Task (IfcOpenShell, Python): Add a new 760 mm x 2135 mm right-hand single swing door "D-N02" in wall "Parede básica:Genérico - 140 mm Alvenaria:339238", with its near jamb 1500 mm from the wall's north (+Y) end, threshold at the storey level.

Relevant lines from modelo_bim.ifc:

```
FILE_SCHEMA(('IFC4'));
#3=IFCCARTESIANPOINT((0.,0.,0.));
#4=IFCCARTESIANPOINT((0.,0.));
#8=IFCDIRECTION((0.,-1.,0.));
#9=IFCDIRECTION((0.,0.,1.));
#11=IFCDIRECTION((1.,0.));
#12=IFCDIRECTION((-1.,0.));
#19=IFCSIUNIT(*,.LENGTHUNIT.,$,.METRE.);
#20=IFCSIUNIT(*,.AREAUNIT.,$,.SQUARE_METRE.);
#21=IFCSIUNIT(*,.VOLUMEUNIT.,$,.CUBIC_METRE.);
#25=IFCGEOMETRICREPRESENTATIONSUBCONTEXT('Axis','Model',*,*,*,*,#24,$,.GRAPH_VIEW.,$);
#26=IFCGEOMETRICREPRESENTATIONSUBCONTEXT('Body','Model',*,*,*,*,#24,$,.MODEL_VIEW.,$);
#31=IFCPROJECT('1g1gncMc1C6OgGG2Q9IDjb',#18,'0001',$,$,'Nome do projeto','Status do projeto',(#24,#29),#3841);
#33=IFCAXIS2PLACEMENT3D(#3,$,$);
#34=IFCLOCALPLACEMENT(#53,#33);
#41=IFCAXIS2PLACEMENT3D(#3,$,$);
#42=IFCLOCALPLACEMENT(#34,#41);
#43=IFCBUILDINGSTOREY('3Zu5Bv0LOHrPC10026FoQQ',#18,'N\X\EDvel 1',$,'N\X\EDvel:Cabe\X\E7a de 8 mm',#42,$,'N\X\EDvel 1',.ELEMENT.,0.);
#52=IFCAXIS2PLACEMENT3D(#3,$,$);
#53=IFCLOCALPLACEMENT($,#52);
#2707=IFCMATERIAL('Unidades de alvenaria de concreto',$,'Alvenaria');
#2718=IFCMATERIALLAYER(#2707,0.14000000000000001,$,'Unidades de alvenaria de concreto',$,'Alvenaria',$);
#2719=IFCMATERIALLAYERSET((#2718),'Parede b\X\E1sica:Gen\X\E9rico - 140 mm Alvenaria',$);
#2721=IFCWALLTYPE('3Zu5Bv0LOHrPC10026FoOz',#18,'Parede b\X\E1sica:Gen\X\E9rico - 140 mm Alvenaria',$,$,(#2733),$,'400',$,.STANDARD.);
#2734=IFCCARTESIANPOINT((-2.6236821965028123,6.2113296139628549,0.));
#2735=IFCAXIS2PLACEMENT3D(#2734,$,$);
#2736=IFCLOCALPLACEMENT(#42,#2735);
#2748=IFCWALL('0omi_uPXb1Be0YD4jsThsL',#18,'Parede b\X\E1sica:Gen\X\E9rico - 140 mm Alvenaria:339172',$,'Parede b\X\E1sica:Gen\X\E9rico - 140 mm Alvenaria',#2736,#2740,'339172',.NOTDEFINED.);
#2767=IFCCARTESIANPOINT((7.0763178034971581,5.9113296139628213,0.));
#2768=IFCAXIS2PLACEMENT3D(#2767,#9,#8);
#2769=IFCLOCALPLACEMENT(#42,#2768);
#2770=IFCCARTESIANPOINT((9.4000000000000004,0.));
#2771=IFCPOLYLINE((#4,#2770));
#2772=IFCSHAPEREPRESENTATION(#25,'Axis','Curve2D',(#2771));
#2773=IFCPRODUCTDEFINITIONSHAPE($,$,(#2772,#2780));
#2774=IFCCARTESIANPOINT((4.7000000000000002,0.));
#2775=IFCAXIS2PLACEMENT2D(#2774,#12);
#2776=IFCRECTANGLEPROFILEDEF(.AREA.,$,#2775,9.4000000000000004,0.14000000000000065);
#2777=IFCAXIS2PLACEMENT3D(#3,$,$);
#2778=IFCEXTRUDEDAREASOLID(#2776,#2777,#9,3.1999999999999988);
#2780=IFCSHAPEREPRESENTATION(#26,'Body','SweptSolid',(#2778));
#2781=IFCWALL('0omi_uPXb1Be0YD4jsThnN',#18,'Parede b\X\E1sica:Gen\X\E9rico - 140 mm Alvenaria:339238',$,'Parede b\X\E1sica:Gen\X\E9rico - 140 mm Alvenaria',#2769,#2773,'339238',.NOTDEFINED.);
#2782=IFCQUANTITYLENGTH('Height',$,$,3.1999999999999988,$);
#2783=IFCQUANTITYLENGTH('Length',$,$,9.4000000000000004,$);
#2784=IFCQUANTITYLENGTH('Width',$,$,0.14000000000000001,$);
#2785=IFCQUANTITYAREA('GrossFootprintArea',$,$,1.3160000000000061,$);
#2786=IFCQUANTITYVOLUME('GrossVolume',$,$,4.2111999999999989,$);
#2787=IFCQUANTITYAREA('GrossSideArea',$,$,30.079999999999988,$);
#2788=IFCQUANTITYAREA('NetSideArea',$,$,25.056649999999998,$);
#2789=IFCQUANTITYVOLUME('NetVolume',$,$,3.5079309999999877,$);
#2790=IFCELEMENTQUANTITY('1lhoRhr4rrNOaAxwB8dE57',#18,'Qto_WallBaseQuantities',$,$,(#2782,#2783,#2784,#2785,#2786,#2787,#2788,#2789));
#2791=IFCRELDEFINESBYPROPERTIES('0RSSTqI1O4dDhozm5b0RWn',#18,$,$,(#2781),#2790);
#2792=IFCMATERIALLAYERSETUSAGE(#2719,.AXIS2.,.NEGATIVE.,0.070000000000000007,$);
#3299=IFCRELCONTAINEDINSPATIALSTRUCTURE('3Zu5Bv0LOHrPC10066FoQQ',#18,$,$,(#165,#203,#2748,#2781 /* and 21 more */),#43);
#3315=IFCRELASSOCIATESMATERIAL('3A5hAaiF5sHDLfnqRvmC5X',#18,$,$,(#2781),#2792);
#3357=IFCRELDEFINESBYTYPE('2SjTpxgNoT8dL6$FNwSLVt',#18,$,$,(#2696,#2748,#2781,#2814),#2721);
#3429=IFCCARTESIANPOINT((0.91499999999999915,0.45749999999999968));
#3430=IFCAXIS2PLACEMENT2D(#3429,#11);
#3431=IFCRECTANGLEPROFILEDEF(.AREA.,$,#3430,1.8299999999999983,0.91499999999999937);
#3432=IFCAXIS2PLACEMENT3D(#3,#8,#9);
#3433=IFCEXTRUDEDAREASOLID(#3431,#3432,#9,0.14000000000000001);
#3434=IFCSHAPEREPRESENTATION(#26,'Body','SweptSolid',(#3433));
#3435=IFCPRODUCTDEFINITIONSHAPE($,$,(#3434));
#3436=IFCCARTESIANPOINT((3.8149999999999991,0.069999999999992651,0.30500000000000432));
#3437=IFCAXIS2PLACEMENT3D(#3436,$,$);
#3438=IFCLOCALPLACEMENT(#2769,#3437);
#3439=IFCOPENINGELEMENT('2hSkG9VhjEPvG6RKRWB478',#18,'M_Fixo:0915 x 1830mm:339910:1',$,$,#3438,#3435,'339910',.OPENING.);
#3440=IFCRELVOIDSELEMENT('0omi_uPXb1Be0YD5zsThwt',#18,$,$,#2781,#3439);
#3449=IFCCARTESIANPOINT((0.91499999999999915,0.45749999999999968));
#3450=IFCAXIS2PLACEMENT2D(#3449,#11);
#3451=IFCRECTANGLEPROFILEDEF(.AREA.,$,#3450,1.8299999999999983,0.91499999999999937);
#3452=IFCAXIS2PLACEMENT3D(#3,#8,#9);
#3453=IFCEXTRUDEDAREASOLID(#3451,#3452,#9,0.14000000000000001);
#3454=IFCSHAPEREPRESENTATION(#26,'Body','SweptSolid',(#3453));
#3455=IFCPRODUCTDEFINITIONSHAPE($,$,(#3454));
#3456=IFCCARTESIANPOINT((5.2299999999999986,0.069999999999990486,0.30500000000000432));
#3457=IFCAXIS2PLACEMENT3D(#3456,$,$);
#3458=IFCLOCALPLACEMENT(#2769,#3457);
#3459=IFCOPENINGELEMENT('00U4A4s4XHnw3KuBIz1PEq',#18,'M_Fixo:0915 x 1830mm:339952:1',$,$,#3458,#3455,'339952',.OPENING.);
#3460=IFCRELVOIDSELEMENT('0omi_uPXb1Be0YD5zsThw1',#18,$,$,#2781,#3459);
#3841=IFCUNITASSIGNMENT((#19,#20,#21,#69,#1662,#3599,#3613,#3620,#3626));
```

```python
import numpy as np
import ifcopenshell
import ifcopenshell.api.feature
import ifcopenshell.api.geometry
import ifcopenshell.api.pset
import ifcopenshell.api.root
import ifcopenshell.api.spatial
import ifcopenshell.geom
import ifcopenshell.util.element
import ifcopenshell.util.placement
import ifcopenshell.util.representation
import ifcopenshell.util.shape
import ifcopenshell.util.unit

model = ifcopenshell.open("modelo_bim.ifc")
unit_scale = ifcopenshell.util.unit.calculate_unit_scale(model)
area_scale = ifcopenshell.util.unit.calculate_unit_scale(model, "AREAUNIT")
volume_scale = ifcopenshell.util.unit.calculate_unit_scale(model, "VOLUMEUNIT")
settings = ifcopenshell.geom.settings()


def volume(element):
    """Net volume in cubic metres, openings subtracted."""
    shape = ifcopenshell.geom.create_shape(settings, element)
    return ifcopenshell.util.shape.get_volume(shape.geometry)


wall = model.by_guid("0omi_uPXb1Be0YD4jsThnN")
storey = ifcopenshell.util.element.get_container(wall, ifc_class="IfcBuildingStorey")
context = ifcopenshell.util.representation.get_context(model, "Model", "Body", "MODEL_VIEW")
before = volume(wall)

width, height, from_end, sill = 0.76, 2.135, 1.5, 0.0  # metres

# The wall runs along its own X axis, and the end named is its -X end.
wall_shape = ifcopenshell.geom.create_shape(settings, wall)
x, y, z = ifcopenshell.util.shape.get_vertices(wall_shape.geometry).T
start = x.min() + from_end
face, thickness = float(y.min()), float(y.max() - y.min())
wall_matrix = ifcopenshell.util.placement.get_local_placement(wall.ObjectPlacement)
level = ifcopenshell.util.placement.get_local_placement(storey.ObjectPlacement)[2, 3]


def in_wall(x, y):
    """Placement at x, y metres in the wall's axes, at sill height."""
    matrix = wall_matrix.copy()
    matrix[:, 3] = wall_matrix @ np.array([x / unit_scale, y / unit_scale, 0.0, 1.0])
    matrix[2, 3] = level + sill / unit_scale
    return matrix


# Opening: a box that overshoots both wall faces by 50 mm.
opening = ifcopenshell.api.root.create_entity(model, ifc_class="IfcOpeningElement", predefined_type="OPENING")
box = ifcopenshell.api.geometry.add_wall_representation(
    model, context=context, length=width, height=height, thickness=thickness + 0.1
)
ifcopenshell.api.geometry.assign_representation(model, product=opening, representation=box)
ifcopenshell.api.geometry.edit_object_placement(model, product=opening, matrix=in_wall(start, face - 0.05), is_si=False)
ifcopenshell.api.feature.add_feature(model, feature=opening, element=wall)

door = ifcopenshell.api.root.create_entity(model, ifc_class="IfcDoor", name="D-N02", predefined_type="DOOR")
door.OverallWidth, door.OverallHeight = width / unit_scale, height / unit_scale
door.OperationType = "SINGLE_SWING_RIGHT"
body = ifcopenshell.api.geometry.add_door_representation(
    model,
    context=context,
    overall_width=door.OverallWidth,
    overall_height=door.OverallHeight,
    operation_type="SINGLE_SWING_RIGHT",
    lining_properties={"LiningDepth": thickness / unit_scale, "ThresholdDepth": thickness / unit_scale},
)
ifcopenshell.api.geometry.assign_representation(model, product=door, representation=body)
ifcopenshell.api.spatial.assign_container(model, products=[door], relating_structure=storey)
ifcopenshell.api.feature.add_filling(model, opening=opening, element=door)

# The lining spans the wall, so the door starts at the wall face.
ifcopenshell.api.geometry.edit_object_placement(model, product=door, matrix=in_wall(start, face), is_si=False)

after = volume(wall)

# Update the wall's stored quantities.
qto = model.by_id(ifcopenshell.util.element.get_pset(wall, "Qto_WallBaseQuantities", should_inherit=False)["id"])
ifcopenshell.api.pset.edit_qto(model, qto=qto, properties={
    "NetSideArea": after / thickness / area_scale,
    "NetVolume": after / volume_scale,
})

print(f"wall volume {before:.3f} -> {after:.3f} m3")

model.write("modelo_bim-out.ifc")
```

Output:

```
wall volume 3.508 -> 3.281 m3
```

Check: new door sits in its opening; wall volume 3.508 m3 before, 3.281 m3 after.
